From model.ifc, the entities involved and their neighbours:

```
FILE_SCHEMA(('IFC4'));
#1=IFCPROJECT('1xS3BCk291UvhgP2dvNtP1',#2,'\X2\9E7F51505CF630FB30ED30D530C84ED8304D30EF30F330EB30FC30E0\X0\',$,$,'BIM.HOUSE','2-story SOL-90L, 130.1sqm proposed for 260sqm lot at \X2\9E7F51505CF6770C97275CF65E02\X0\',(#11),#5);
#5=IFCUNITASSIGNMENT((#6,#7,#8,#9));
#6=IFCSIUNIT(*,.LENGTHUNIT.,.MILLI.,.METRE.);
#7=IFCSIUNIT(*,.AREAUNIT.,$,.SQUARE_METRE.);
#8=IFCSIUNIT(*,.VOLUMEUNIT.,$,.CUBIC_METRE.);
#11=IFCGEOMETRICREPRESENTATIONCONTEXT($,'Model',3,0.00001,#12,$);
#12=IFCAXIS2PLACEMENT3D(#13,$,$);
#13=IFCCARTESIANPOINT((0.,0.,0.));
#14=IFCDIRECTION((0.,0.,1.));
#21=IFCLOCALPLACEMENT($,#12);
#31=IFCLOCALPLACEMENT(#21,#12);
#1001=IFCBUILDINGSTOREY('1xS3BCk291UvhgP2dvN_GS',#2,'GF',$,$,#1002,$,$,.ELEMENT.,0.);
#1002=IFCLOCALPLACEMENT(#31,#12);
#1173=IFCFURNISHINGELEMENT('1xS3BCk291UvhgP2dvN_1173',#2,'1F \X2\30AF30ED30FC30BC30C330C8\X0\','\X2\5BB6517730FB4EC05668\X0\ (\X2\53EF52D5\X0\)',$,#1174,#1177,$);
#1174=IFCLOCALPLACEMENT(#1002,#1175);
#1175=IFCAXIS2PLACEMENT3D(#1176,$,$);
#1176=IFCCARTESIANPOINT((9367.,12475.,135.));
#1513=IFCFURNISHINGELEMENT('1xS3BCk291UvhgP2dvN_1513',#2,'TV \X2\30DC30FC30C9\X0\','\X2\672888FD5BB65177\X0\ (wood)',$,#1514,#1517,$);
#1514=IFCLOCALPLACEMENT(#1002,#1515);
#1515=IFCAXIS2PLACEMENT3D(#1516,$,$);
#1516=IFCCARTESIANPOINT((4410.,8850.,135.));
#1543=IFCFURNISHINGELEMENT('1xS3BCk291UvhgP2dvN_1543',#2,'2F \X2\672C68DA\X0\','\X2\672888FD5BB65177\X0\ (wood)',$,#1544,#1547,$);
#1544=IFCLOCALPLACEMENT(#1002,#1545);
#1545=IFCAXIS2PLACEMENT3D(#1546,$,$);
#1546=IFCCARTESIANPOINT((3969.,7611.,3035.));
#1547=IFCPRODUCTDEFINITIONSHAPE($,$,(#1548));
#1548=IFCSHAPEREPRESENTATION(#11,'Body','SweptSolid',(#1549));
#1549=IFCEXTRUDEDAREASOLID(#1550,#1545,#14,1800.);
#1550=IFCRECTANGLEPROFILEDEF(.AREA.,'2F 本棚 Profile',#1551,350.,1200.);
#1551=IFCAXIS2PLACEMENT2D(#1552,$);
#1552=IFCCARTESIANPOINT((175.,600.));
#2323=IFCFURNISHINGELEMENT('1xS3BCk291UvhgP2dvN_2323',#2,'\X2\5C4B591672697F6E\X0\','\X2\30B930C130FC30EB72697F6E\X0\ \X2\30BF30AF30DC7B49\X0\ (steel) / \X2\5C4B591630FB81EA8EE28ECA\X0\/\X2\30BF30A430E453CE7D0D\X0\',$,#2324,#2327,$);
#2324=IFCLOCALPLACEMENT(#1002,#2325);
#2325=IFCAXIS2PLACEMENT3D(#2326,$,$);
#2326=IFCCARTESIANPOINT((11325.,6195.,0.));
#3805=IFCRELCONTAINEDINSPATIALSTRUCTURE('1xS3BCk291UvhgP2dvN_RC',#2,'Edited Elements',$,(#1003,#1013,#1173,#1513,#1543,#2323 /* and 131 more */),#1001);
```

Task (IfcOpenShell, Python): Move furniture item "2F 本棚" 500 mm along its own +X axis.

```python
import ifcopenshell
import ifcopenshell.api.geometry
import ifcopenshell.util.placement
import ifcopenshell.util.unit

model = ifcopenshell.open("model.ifc")
unit_scale = ifcopenshell.util.unit.calculate_unit_scale(model)

item = model.by_id(1543)
matrix = ifcopenshell.util.placement.get_local_placement(item.ObjectPlacement)
matrix[:3, 3] += matrix[:3, 0] * 0.5 / unit_scale
ifcopenshell.api.geometry.edit_object_placement(model, product=item, matrix=matrix, is_si=False)

print(ifcopenshell.util.placement.get_local_placement(item.ObjectPlacement).round(3) + 0.0)

model.write("model_v2.ifc")
```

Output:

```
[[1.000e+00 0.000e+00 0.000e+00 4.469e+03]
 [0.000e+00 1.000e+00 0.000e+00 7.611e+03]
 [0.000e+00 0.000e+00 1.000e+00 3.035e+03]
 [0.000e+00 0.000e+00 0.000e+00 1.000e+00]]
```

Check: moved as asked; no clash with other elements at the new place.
